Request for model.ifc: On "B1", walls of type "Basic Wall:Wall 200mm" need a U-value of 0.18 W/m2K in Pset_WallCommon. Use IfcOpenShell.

First a look at what the model holds.

```python
import ifcopenshell
import ifcopenshell.util.element

model = ifcopenshell.open("model.ifc")
print(model.schema)
storey = next(s for s in model.by_type("IfcBuildingStorey") if s.Name == "B1")
walls = [e for e in ifcopenshell.util.element.get_decomposition(storey) if e.is_a("IfcWall")]
seen = {}
for e in walls:
    element_type = ifcopenshell.util.element.get_type(e)
    key = (element_type.Name if element_type != e and element_type else None, ifcopenshell.util.element.get_pset(e, "Pset_WallCommon", "ThermalTransmittance"))
    seen[key] = seen.get(key, 0) + 1
for (name, value), count in sorted(seen.items(), key=str):
    print(count, "x", name, "|", value)
```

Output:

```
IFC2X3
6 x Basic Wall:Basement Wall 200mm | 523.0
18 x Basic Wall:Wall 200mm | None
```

```python
import ifcopenshell
import ifcopenshell.api.pset
import ifcopenshell.util.element

model = ifcopenshell.open("model.ifc")

storey = next(s for s in model.by_type("IfcBuildingStorey") if s.Name == "B1")
walls = [e for e in ifcopenshell.util.element.get_decomposition(storey) if e.is_a("IfcWall")]

count = 0
for e in walls:
    element_type = ifcopenshell.util.element.get_type(e)
    if element_type in (None, e) or element_type.Name != "Basic Wall:Wall 200mm":
        continue
    # add_pset returns the element's existing set when there is one.
    pset = ifcopenshell.api.pset.add_pset(model, product=e, name="Pset_WallCommon")
    ifcopenshell.api.pset.edit_pset(model, pset=pset, properties={"ThermalTransmittance": 0.18})
    count += 1

print(count, "walls updated")

model.write("model-out.ifc")
```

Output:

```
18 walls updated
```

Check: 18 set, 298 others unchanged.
